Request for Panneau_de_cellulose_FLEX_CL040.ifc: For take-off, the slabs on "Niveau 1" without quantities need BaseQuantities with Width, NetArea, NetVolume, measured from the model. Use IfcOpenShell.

First a look at what the model holds.

```python
import ifcopenshell
import ifcopenshell.util.element
import ifcopenshell.util.unit

model = ifcopenshell.open("Panneau_de_cellulose_FLEX_CL040.ifc")
print(model.schema)
for unit_type in ("LENGTHUNIT", "AREAUNIT", "VOLUMEUNIT"):
    print(unit_type, ifcopenshell.util.unit.calculate_unit_scale(model, unit_type))
storey = next(s for s in model.by_type("IfcBuildingStorey") if s.Name == "Niveau 1")
slabs = [e for e in ifcopenshell.util.element.get_decomposition(storey) if e.is_a("IfcSlab")]
for e in sorted(slabs, key=lambda e: e.id()):
    print(e.id(), e.is_a(), e.Name, list(ifcopenshell.util.element.get_psets(e, qtos_only=True)), sep=" | ")
```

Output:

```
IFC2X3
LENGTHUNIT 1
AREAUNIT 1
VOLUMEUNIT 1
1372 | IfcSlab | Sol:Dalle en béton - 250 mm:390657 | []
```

```python
import ifcopenshell
import ifcopenshell.api.pset
import ifcopenshell.geom
import ifcopenshell.util.element
import ifcopenshell.util.shape
import ifcopenshell.util.unit

model = ifcopenshell.open("Panneau_de_cellulose_FLEX_CL040.ifc")
unit_scale = ifcopenshell.util.unit.calculate_unit_scale(model)
area_scale = ifcopenshell.util.unit.calculate_unit_scale(model, "AREAUNIT")
volume_scale = ifcopenshell.util.unit.calculate_unit_scale(model, "VOLUMEUNIT")
settings = ifcopenshell.geom.settings()

storey = next(s for s in model.by_type("IfcBuildingStorey") if s.Name == "Niveau 1")
slabs = [e for e in ifcopenshell.util.element.get_decomposition(storey) if e.is_a("IfcSlab")]

for e in sorted(slabs, key=lambda e: e.id()):
    if ifcopenshell.util.element.get_psets(e, qtos_only=True, should_inherit=False):
        continue
    # Geometry comes back in metres, in the element's own axes.
    shape = ifcopenshell.geom.create_shape(settings, e)
    values = {
        "Width": ifcopenshell.util.shape.get_z(shape.geometry) / unit_scale,
        "NetArea": ifcopenshell.util.shape.get_footprint_area(shape.geometry) / area_scale,
        "NetVolume": ifcopenshell.util.shape.get_volume(shape.geometry) / volume_scale,
    }
    qto = ifcopenshell.api.pset.add_qto(model, product=e, name="BaseQuantities")
    ifcopenshell.api.pset.edit_qto(model, qto=qto, properties=values)
    print(e.id(), {k: round(v, 3) for k, v in values.items()})

model.write("Panneau_de_cellulose_FLEX_CL040_edited.ifc")
```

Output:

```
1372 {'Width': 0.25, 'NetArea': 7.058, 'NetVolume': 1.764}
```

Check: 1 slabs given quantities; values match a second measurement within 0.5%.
